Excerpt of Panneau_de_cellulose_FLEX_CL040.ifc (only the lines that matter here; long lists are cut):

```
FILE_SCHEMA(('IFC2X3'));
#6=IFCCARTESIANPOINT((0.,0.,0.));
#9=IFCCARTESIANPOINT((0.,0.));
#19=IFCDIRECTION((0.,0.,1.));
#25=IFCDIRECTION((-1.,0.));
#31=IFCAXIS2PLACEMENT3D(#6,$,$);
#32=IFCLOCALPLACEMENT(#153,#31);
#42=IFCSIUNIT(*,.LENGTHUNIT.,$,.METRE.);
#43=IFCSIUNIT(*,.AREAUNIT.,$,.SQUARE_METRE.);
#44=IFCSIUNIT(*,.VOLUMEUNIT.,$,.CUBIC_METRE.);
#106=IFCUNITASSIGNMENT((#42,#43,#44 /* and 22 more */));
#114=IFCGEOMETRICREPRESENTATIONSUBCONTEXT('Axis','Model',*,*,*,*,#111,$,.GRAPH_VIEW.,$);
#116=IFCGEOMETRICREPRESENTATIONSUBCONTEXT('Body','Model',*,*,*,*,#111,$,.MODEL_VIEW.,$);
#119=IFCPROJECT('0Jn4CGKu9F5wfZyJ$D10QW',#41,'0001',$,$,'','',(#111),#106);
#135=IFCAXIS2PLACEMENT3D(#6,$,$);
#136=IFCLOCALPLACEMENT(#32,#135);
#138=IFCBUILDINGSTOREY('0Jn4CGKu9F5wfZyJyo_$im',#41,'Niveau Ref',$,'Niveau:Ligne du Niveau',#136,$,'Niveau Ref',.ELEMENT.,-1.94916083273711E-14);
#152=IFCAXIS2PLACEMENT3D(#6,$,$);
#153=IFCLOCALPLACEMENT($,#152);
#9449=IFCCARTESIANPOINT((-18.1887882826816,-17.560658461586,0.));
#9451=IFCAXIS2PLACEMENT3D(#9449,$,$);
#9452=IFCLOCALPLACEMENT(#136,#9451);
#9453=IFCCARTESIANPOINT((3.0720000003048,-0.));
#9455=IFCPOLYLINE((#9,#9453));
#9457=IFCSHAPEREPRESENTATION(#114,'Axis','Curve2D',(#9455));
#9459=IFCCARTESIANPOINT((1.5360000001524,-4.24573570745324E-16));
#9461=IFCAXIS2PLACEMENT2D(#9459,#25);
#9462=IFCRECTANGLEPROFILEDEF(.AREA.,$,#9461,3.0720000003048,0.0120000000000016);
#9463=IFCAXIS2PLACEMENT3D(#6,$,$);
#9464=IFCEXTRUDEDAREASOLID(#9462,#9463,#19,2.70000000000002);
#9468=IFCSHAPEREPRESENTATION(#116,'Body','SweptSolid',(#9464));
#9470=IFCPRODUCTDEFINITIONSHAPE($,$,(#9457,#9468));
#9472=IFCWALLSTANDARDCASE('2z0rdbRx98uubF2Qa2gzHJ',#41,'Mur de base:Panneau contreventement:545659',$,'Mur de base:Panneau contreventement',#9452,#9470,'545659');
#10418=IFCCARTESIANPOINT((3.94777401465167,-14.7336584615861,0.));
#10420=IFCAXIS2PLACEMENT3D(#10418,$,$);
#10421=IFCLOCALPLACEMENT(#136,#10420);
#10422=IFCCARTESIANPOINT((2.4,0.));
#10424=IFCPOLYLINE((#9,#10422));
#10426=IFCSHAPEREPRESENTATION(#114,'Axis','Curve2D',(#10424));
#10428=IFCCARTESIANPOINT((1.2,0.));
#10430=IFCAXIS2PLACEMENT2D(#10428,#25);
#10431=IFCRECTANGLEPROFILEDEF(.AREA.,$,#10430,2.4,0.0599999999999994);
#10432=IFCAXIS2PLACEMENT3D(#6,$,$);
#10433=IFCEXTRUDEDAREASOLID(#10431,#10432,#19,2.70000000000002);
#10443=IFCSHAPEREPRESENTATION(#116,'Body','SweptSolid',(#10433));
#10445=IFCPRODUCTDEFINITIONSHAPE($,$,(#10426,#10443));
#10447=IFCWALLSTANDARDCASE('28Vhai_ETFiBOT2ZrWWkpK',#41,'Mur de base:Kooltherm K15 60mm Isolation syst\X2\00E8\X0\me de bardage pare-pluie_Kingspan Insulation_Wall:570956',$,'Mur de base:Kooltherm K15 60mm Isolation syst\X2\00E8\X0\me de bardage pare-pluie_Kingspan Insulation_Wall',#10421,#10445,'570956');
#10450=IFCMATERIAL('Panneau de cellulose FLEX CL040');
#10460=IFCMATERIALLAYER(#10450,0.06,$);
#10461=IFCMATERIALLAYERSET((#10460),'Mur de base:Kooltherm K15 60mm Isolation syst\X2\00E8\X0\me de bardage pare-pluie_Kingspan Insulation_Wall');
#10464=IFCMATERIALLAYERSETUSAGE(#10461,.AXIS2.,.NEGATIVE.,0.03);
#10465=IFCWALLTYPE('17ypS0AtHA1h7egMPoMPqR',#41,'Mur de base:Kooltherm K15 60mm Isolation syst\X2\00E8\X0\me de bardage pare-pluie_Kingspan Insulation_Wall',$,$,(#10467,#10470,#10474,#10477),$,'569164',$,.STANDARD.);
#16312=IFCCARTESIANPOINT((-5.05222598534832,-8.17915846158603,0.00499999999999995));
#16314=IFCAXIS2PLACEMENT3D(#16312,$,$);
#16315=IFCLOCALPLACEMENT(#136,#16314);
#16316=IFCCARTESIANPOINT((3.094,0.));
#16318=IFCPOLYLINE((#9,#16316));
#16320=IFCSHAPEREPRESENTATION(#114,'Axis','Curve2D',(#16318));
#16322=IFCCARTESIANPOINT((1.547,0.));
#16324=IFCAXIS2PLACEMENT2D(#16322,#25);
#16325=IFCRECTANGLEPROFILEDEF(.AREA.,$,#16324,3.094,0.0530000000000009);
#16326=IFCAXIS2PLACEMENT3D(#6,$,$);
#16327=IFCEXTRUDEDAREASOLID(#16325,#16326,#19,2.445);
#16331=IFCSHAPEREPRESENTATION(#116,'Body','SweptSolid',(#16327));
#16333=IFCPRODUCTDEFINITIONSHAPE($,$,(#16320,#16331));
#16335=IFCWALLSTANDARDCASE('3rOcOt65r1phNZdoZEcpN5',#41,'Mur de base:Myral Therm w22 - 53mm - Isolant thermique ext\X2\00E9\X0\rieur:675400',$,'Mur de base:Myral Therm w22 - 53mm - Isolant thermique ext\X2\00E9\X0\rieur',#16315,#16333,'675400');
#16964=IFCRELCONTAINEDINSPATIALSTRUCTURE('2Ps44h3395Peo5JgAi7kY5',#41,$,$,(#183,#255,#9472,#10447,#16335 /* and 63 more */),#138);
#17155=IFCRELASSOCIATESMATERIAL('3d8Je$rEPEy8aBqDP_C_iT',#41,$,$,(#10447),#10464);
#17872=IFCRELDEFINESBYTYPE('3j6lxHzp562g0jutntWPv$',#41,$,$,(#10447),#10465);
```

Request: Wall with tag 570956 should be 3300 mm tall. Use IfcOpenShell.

```python
import ifcopenshell
import ifcopenshell.geom
import ifcopenshell.util.representation
import ifcopenshell.util.shape
import ifcopenshell.util.unit

model = ifcopenshell.open("Panneau_de_cellulose_FLEX_CL040.ifc")
unit_scale = ifcopenshell.util.unit.calculate_unit_scale(model)
settings = ifcopenshell.geom.settings()


def volume(element):
    """Net volume in cubic metres, openings subtracted."""
    shape = ifcopenshell.geom.create_shape(settings, element)
    return ifcopenshell.util.shape.get_volume(shape.geometry)


wall = model.by_guid("28Vhai_ETFiBOT2ZrWWkpK")
before = volume(wall)

body = ifcopenshell.util.representation.get_representation(wall, "Model", "Body")
solid = body.Items[0]
old_height = solid.Depth
solid.Depth = 3.3 / unit_scale
after = volume(wall)

print(f"height {old_height:g} -> {solid.Depth:g}, volume {before:.3f} -> {after:.3f} m3")

model.write("Panneau_de_cellulose_FLEX_CL040_edited.ifc")
```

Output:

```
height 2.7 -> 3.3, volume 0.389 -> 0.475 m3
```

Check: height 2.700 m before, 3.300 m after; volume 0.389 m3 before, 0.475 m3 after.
